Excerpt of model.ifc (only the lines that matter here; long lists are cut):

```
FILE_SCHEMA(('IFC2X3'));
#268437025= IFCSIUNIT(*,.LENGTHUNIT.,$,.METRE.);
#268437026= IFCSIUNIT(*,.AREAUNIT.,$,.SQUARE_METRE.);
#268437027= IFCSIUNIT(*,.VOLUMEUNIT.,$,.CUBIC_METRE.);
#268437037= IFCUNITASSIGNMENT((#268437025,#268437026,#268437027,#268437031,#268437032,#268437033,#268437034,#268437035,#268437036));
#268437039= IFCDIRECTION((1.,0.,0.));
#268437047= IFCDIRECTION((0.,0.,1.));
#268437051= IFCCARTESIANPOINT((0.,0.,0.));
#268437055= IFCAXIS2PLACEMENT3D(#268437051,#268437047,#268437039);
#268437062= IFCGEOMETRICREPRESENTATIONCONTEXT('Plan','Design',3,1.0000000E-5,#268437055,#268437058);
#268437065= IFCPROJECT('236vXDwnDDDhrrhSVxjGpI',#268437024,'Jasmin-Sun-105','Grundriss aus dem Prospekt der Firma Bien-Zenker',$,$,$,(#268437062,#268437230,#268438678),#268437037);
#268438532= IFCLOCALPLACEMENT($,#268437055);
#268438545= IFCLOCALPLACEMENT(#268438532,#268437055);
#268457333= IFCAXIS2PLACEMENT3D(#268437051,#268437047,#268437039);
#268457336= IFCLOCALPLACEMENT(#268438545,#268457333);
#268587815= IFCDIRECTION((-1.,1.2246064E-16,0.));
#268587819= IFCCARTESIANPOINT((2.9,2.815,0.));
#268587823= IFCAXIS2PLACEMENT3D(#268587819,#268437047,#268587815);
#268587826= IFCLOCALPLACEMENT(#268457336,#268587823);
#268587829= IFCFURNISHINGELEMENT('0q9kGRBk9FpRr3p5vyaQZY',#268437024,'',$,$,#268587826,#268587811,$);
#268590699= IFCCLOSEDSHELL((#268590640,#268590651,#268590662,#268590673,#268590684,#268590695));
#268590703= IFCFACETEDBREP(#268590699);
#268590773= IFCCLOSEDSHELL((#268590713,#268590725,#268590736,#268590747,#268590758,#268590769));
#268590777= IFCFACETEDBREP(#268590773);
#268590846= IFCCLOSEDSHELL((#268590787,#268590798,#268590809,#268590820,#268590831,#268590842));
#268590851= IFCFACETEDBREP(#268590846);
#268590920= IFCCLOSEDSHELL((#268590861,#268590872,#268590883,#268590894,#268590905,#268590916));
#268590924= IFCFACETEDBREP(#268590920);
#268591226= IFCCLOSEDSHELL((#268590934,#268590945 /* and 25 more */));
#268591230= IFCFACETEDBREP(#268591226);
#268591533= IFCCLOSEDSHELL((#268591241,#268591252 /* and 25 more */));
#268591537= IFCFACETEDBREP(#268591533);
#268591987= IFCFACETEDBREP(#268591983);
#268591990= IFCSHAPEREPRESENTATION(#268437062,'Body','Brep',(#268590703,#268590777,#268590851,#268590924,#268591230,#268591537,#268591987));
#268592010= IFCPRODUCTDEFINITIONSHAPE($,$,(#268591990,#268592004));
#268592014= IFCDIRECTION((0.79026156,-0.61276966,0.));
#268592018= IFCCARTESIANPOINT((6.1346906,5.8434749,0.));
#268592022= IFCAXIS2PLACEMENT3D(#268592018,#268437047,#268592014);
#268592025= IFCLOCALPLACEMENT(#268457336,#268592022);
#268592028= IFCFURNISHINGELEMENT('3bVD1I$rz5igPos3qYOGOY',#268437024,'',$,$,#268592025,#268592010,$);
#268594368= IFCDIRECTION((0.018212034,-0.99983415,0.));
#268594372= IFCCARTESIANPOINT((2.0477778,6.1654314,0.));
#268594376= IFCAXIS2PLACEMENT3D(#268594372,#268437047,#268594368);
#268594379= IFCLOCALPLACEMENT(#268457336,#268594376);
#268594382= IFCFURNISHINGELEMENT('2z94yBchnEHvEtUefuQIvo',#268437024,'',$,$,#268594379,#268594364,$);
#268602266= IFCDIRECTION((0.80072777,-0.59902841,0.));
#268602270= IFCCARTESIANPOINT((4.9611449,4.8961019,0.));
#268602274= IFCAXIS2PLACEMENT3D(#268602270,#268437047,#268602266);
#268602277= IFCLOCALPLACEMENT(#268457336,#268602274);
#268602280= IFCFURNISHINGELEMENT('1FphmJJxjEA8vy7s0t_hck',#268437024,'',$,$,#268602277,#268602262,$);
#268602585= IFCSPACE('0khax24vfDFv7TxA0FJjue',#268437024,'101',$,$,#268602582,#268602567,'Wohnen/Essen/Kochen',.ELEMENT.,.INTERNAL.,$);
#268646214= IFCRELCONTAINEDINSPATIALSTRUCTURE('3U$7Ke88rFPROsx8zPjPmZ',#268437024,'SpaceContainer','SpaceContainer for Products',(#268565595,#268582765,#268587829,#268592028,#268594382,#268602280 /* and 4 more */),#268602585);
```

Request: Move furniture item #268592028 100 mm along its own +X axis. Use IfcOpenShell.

```python
import ifcopenshell
import ifcopenshell.api.geometry
import ifcopenshell.util.placement
import ifcopenshell.util.unit

model = ifcopenshell.open("model.ifc")
unit_scale = ifcopenshell.util.unit.calculate_unit_scale(model)

item = model.by_guid("3bVD1I$rz5igPos3qYOGOY")
matrix = ifcopenshell.util.placement.get_local_placement(item.ObjectPlacement)
matrix[:3, 3] += matrix[:3, 0] * 0.1 / unit_scale
ifcopenshell.api.geometry.edit_object_placement(model, product=item, matrix=matrix, is_si=False)

print(ifcopenshell.util.placement.get_local_placement(item.ObjectPlacement).round(3) + 0.0)

model.write("model_rev.ifc")
```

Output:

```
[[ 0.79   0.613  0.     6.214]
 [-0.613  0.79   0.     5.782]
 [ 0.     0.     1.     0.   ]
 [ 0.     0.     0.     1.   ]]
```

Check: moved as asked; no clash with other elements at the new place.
